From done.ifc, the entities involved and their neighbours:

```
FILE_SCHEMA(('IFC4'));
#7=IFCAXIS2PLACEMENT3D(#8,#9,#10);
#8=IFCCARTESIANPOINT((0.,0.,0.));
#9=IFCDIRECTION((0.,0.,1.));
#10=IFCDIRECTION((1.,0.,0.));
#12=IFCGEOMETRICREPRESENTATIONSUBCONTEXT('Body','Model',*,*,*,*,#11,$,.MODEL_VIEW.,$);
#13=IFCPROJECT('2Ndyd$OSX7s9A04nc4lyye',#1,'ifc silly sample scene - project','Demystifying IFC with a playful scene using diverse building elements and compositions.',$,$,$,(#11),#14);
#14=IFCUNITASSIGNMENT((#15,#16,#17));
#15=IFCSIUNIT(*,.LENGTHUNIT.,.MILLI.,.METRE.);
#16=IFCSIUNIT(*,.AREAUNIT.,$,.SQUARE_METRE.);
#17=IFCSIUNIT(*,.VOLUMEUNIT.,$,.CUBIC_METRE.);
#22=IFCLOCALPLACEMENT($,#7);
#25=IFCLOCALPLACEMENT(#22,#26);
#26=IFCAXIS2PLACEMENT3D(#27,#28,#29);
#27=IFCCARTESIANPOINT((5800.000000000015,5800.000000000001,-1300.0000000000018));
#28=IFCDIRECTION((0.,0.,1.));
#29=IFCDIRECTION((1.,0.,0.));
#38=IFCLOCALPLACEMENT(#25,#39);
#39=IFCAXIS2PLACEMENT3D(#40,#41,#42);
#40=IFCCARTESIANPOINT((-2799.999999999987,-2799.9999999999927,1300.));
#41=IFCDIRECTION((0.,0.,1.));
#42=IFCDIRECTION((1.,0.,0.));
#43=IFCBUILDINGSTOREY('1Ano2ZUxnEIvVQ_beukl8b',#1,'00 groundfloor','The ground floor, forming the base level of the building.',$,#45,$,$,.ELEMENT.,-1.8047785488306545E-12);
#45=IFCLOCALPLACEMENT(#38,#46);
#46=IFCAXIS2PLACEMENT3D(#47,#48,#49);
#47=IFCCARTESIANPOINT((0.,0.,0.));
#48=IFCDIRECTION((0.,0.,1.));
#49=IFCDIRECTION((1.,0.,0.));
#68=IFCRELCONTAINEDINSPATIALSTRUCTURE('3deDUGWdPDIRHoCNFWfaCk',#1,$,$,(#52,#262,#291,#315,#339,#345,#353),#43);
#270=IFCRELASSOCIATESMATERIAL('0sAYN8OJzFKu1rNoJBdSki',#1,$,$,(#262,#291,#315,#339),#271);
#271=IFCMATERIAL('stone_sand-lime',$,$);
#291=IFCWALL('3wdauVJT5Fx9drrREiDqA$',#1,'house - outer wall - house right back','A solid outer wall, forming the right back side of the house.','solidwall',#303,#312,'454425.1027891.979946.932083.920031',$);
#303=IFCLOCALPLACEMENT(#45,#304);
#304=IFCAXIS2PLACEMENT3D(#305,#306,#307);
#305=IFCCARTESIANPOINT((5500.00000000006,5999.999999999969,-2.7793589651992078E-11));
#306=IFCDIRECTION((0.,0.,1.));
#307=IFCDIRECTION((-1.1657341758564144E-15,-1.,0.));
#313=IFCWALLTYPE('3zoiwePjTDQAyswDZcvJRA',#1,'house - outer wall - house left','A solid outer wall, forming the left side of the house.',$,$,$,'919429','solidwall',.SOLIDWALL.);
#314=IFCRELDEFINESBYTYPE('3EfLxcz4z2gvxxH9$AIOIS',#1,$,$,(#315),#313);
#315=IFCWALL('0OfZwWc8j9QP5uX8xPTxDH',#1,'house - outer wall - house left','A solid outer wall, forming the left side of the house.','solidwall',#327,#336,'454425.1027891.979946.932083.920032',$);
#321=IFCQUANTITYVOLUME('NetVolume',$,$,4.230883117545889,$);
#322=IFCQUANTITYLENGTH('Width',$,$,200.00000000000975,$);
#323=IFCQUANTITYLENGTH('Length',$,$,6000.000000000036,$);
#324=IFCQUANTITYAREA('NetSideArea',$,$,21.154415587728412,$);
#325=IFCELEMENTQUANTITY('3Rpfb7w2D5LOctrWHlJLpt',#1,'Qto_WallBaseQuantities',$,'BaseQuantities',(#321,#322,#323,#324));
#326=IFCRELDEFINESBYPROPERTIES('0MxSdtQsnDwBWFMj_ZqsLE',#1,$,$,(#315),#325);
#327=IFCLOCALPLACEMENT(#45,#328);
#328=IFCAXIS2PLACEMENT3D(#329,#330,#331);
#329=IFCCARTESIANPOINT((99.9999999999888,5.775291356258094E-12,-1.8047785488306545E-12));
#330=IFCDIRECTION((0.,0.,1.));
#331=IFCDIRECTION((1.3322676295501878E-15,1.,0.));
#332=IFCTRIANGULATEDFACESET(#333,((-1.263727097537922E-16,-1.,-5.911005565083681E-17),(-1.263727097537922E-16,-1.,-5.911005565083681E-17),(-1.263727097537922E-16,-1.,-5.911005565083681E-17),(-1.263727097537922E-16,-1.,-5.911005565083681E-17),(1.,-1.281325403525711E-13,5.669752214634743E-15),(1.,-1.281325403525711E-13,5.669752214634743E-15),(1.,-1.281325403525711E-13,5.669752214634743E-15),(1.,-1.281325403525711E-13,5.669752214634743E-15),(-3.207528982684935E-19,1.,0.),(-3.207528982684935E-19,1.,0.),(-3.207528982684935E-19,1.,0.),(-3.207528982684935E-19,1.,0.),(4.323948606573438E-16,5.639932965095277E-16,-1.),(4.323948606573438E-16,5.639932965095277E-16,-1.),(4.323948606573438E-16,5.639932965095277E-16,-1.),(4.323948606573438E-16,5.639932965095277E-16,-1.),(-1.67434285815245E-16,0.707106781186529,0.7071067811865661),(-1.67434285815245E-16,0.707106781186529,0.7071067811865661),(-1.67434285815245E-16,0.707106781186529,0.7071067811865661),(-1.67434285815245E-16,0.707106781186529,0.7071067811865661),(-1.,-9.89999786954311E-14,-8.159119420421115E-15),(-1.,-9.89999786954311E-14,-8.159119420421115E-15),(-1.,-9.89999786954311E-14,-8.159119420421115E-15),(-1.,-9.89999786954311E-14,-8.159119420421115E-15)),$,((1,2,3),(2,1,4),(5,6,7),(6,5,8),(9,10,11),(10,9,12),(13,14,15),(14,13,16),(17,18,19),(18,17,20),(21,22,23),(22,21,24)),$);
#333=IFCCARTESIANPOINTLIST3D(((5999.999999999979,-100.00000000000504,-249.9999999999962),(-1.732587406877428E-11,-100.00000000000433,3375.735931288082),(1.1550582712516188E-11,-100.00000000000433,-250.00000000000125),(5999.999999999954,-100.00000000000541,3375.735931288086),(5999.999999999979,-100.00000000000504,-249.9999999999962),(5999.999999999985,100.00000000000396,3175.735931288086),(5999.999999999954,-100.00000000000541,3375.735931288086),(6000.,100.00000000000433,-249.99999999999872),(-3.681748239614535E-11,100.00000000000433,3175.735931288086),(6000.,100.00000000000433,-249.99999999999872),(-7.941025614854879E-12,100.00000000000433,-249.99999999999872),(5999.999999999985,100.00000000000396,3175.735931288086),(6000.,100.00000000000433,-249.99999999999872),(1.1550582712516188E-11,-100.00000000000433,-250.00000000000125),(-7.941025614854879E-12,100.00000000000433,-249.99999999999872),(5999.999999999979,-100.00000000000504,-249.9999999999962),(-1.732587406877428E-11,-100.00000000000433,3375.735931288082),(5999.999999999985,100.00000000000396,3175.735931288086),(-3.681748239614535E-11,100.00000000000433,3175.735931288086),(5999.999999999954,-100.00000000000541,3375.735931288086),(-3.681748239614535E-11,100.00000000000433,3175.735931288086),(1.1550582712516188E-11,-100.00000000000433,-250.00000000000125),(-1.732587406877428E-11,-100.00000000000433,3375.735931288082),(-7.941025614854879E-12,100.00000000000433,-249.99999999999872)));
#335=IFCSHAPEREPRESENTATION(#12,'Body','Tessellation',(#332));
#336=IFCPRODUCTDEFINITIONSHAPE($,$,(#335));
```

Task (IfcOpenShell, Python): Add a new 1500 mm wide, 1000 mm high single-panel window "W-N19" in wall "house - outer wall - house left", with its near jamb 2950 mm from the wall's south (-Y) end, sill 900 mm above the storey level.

```python
import numpy as np
import ifcopenshell
import ifcopenshell.api.feature
import ifcopenshell.api.geometry
import ifcopenshell.api.pset
import ifcopenshell.api.root
import ifcopenshell.api.spatial
import ifcopenshell.geom
import ifcopenshell.util.element
import ifcopenshell.util.placement
import ifcopenshell.util.representation
import ifcopenshell.util.shape
import ifcopenshell.util.unit

model = ifcopenshell.open("done.ifc")
unit_scale = ifcopenshell.util.unit.calculate_unit_scale(model)
area_scale = ifcopenshell.util.unit.calculate_unit_scale(model, "AREAUNIT")
volume_scale = ifcopenshell.util.unit.calculate_unit_scale(model, "VOLUMEUNIT")
settings = ifcopenshell.geom.settings()


def volume(element):
    """Net volume in cubic metres, openings subtracted."""
    shape = ifcopenshell.geom.create_shape(settings, element)
    return ifcopenshell.util.shape.get_volume(shape.geometry)


wall = model.by_id(315)
storey = ifcopenshell.util.element.get_container(wall, ifc_class="IfcBuildingStorey")
context = ifcopenshell.util.representation.get_context(model, "Model", "Body", "MODEL_VIEW")
before = volume(wall)

width, height, from_end, sill = 1.5, 1, 2.95, 0.9  # metres

# The wall runs along its own X axis, and the end named is its -X end.
wall_shape = ifcopenshell.geom.create_shape(settings, wall)
x, y, z = ifcopenshell.util.shape.get_vertices(wall_shape.geometry).T
start = x.min() + from_end
face, thickness = float(y.min()), float(y.max() - y.min())
wall_matrix = ifcopenshell.util.placement.get_local_placement(wall.ObjectPlacement)
level = ifcopenshell.util.placement.get_local_placement(storey.ObjectPlacement)[2, 3]


def in_wall(x, y):
    """Placement at x, y metres in the wall's axes, at sill height."""
    matrix = wall_matrix.copy()
    matrix[:, 3] = wall_matrix @ np.array([x / unit_scale, y / unit_scale, 0.0, 1.0])
    matrix[2, 3] = level + sill / unit_scale
    return matrix


# Opening: a box that overshoots both wall faces by 50 mm.
opening = ifcopenshell.api.root.create_entity(model, ifc_class="IfcOpeningElement", predefined_type="OPENING")
box = ifcopenshell.api.geometry.add_wall_representation(
    model, context=context, length=width, height=height, thickness=thickness + 0.1
)
ifcopenshell.api.geometry.assign_representation(model, product=opening, representation=box)
ifcopenshell.api.geometry.edit_object_placement(model, product=opening, matrix=in_wall(start, face - 0.05), is_si=False)
ifcopenshell.api.feature.add_feature(model, feature=opening, element=wall)

window = ifcopenshell.api.root.create_entity(model, ifc_class="IfcWindow", name="W-N19", predefined_type="WINDOW")
window.OverallWidth, window.OverallHeight = width / unit_scale, height / unit_scale
window.PartitioningType = "SINGLE_PANEL"
body = ifcopenshell.api.geometry.add_window_representation(
    model,
    context=context,
    overall_width=window.OverallWidth,
    overall_height=window.OverallHeight,
    partition_type="SINGLE_PANEL",
)
ifcopenshell.api.geometry.assign_representation(model, product=window, representation=body)
ifcopenshell.api.spatial.assign_container(model, products=[window], relating_structure=storey)
ifcopenshell.api.feature.add_filling(model, opening=opening, element=window)

# Centre the window in the wall's thickness.
ifcopenshell.api.geometry.edit_object_placement(model, product=window, matrix=in_wall(start, face), is_si=False)
window_shape = ifcopenshell.geom.create_shape(settings, window)
depth = ifcopenshell.util.shape.get_vertices(window_shape.geometry)[:, 1]
offset = face + thickness / 2 - (depth.min() + depth.max()) / 2
ifcopenshell.api.geometry.edit_object_placement(model, product=window, matrix=in_wall(start, offset), is_si=False)

after = volume(wall)

# Update the wall's stored quantities.
qto = model.by_id(ifcopenshell.util.element.get_pset(wall, "Qto_WallBaseQuantities", should_inherit=False)["id"])
ifcopenshell.api.pset.edit_qto(model, qto=qto, properties={
    "NetVolume": after / volume_scale,
    "NetSideArea": after / thickness / area_scale,
})

print(f"wall volume {before:.3f} -> {after:.3f} m3")

model.write("done-out.ifc")
```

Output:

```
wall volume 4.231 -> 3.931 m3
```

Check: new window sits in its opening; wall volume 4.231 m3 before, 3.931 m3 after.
